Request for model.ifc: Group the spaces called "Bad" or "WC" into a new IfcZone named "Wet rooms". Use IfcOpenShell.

First a look at what the model holds.

```python
import ifcopenshell

model = ifcopenshell.open("model.ifc")
print(model.schema)
seen = {}
for space in model.by_type("IfcSpace"):
    seen[space.LongName] = seen.get(space.LongName, 0) + 1
for name, count in sorted(seen.items(), key=str):
    print(count, "x", name)
print("zones:", [z.Name for z in model.by_type("IfcZone")][:20])
```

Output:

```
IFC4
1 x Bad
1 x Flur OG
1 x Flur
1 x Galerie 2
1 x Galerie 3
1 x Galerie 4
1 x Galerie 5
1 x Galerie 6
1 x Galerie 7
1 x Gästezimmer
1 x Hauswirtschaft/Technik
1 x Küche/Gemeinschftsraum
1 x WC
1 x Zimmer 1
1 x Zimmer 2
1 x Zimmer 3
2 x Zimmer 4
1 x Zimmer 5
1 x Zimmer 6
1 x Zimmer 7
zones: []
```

```python
import ifcopenshell
import ifcopenshell.api.group
import ifcopenshell.api.root

model = ifcopenshell.open("model.ifc")

names = {"Bad", "WC"}
spaces = [s for s in model.by_type("IfcSpace") if s.LongName in names]

zone = ifcopenshell.api.root.create_entity(model, ifc_class="IfcZone", name="Wet rooms")
ifcopenshell.api.group.assign_group(model, products=spaces, group=zone)
print(len(spaces), "spaces in", zone.Name)

model.write("model_updated.ifc")
```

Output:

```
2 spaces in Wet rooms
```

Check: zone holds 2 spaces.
